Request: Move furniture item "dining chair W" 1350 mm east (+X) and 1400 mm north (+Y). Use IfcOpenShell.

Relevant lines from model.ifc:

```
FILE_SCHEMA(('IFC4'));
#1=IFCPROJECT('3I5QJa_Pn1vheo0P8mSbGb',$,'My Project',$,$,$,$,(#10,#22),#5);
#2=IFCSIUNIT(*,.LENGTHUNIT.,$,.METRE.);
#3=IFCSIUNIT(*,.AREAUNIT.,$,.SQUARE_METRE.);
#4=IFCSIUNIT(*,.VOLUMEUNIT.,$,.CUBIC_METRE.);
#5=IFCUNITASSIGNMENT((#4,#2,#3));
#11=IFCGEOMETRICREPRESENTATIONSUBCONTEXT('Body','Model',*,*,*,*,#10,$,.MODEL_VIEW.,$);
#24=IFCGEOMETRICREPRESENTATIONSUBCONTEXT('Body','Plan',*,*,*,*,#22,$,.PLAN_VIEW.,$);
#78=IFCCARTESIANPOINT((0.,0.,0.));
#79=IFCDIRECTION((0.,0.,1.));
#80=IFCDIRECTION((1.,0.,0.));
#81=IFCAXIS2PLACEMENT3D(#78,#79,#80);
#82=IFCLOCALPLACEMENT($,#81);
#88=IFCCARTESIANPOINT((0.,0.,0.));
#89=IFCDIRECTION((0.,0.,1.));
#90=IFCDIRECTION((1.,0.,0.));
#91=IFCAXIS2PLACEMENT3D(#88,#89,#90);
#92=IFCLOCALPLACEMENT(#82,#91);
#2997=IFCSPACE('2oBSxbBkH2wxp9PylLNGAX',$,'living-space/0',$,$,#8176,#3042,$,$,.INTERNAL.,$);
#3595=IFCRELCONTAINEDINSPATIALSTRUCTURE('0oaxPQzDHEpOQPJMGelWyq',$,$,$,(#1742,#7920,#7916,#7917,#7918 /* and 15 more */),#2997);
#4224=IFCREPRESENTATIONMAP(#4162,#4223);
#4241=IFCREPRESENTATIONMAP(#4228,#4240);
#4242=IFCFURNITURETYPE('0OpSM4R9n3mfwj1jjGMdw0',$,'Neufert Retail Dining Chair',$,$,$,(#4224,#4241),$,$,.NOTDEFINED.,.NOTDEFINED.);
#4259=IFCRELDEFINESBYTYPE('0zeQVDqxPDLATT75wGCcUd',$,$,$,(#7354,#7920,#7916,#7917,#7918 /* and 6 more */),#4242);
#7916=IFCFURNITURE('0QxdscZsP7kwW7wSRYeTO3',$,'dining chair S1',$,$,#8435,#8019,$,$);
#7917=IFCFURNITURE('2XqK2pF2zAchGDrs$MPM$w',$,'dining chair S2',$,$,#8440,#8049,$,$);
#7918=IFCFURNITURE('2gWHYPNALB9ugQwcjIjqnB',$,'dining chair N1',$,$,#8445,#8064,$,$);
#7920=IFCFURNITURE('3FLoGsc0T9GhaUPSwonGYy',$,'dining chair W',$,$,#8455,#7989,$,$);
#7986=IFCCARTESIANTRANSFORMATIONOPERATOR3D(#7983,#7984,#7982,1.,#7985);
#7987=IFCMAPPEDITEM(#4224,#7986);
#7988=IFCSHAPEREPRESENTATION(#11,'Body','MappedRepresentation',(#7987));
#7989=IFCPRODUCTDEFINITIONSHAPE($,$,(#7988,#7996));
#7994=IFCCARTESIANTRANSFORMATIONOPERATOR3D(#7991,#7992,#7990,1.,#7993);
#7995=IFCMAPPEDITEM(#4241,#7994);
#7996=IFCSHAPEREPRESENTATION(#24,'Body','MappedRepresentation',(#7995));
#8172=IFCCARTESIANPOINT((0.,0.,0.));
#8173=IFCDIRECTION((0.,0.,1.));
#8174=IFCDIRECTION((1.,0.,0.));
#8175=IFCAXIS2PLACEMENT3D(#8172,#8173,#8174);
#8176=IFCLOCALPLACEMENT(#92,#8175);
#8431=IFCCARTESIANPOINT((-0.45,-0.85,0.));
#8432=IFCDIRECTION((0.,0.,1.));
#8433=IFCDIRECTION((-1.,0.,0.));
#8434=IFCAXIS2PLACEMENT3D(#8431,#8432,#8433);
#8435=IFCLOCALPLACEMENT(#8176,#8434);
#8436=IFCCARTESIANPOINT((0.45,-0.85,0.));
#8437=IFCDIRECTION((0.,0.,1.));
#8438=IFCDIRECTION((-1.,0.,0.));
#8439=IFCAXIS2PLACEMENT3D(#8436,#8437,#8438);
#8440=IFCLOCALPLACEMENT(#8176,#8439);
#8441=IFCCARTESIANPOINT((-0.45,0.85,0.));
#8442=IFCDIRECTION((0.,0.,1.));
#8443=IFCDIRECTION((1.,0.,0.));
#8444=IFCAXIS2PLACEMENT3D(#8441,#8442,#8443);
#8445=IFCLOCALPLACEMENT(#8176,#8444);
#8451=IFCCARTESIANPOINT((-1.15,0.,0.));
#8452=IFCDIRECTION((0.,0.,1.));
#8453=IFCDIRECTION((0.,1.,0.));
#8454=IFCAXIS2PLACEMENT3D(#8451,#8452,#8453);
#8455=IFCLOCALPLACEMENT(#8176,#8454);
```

```python
import ifcopenshell
import ifcopenshell.api.geometry
import ifcopenshell.util.placement
import ifcopenshell.util.unit

model = ifcopenshell.open("model.ifc")
unit_scale = ifcopenshell.util.unit.calculate_unit_scale(model)

item = model.by_guid("3FLoGsc0T9GhaUPSwonGYy")
matrix = ifcopenshell.util.placement.get_local_placement(item.ObjectPlacement)
matrix[0, 3] += 1.35 / unit_scale
matrix[1, 3] += 1.4 / unit_scale
ifcopenshell.api.geometry.edit_object_placement(model, product=item, matrix=matrix, is_si=False)

print(ifcopenshell.util.placement.get_local_placement(item.ObjectPlacement).round(3) + 0.0)

model.write("model_v2.ifc")
```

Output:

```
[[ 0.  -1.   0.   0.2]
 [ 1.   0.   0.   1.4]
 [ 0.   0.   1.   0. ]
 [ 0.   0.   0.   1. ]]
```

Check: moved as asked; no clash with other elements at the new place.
